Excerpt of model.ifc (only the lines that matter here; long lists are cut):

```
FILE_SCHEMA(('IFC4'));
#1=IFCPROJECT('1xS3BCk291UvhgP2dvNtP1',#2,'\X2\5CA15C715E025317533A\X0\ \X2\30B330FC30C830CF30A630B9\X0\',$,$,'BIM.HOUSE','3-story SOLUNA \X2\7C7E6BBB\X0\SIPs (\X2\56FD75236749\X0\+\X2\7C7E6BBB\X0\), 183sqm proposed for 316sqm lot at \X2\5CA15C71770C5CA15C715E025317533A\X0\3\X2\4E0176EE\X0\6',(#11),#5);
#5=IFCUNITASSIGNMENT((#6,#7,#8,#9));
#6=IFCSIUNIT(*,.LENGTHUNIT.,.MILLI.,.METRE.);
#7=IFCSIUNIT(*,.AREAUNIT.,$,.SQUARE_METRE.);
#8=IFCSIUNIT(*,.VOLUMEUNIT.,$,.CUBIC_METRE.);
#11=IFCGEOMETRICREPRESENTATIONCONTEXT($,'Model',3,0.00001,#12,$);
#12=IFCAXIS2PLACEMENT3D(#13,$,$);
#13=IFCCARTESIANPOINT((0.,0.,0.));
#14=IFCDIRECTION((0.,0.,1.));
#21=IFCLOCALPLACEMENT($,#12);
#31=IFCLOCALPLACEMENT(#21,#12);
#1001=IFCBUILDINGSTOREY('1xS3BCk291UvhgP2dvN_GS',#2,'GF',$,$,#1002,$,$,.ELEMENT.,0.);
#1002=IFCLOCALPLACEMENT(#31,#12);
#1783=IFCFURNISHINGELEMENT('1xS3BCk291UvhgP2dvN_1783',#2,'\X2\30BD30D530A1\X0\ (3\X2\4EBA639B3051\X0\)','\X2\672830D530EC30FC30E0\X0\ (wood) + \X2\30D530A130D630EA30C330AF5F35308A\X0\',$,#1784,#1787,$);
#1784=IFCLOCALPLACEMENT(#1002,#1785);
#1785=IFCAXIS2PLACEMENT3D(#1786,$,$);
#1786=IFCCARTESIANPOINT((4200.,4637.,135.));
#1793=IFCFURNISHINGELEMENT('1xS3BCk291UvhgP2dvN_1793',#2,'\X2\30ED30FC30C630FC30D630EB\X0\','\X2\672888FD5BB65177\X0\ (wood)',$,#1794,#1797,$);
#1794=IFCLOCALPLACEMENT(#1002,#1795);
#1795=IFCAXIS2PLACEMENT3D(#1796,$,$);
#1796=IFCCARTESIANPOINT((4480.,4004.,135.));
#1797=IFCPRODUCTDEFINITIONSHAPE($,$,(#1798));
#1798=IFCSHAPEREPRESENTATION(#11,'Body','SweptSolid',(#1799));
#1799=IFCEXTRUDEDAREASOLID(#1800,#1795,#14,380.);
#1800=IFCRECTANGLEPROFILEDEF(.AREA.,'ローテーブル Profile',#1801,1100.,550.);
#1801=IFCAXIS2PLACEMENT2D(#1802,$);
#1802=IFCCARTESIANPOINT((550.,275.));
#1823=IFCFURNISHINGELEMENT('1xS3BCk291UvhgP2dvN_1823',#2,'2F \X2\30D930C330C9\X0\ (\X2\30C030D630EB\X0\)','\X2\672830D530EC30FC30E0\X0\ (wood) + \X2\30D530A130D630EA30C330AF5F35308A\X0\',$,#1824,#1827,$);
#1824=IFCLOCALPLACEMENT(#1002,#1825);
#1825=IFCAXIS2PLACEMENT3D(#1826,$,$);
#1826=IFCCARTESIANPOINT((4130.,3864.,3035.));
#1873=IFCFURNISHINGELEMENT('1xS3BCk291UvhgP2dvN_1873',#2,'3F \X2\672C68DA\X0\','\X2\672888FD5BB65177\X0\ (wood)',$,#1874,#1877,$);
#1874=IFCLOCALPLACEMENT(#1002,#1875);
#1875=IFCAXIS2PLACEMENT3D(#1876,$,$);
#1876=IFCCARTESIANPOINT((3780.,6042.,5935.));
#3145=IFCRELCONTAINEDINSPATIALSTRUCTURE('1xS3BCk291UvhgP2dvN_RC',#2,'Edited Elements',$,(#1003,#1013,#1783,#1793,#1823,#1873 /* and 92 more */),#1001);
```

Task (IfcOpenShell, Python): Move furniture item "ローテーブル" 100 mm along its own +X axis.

```python
import ifcopenshell
import ifcopenshell.api.geometry
import ifcopenshell.util.placement
import ifcopenshell.util.unit

model = ifcopenshell.open("model.ifc")
unit_scale = ifcopenshell.util.unit.calculate_unit_scale(model)

item = model.by_guid("1xS3BCk291UvhgP2dvN_1793")
matrix = ifcopenshell.util.placement.get_local_placement(item.ObjectPlacement)
matrix[:3, 3] += matrix[:3, 0] * 0.1 / unit_scale
ifcopenshell.api.geometry.edit_object_placement(model, product=item, matrix=matrix, is_si=False)

print(ifcopenshell.util.placement.get_local_placement(item.ObjectPlacement).round(3) + 0.0)

model.write("model_updated.ifc")
```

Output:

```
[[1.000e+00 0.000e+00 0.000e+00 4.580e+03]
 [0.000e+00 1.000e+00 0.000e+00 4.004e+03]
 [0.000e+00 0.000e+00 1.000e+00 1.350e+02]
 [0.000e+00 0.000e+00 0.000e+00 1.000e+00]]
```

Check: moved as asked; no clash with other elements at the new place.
